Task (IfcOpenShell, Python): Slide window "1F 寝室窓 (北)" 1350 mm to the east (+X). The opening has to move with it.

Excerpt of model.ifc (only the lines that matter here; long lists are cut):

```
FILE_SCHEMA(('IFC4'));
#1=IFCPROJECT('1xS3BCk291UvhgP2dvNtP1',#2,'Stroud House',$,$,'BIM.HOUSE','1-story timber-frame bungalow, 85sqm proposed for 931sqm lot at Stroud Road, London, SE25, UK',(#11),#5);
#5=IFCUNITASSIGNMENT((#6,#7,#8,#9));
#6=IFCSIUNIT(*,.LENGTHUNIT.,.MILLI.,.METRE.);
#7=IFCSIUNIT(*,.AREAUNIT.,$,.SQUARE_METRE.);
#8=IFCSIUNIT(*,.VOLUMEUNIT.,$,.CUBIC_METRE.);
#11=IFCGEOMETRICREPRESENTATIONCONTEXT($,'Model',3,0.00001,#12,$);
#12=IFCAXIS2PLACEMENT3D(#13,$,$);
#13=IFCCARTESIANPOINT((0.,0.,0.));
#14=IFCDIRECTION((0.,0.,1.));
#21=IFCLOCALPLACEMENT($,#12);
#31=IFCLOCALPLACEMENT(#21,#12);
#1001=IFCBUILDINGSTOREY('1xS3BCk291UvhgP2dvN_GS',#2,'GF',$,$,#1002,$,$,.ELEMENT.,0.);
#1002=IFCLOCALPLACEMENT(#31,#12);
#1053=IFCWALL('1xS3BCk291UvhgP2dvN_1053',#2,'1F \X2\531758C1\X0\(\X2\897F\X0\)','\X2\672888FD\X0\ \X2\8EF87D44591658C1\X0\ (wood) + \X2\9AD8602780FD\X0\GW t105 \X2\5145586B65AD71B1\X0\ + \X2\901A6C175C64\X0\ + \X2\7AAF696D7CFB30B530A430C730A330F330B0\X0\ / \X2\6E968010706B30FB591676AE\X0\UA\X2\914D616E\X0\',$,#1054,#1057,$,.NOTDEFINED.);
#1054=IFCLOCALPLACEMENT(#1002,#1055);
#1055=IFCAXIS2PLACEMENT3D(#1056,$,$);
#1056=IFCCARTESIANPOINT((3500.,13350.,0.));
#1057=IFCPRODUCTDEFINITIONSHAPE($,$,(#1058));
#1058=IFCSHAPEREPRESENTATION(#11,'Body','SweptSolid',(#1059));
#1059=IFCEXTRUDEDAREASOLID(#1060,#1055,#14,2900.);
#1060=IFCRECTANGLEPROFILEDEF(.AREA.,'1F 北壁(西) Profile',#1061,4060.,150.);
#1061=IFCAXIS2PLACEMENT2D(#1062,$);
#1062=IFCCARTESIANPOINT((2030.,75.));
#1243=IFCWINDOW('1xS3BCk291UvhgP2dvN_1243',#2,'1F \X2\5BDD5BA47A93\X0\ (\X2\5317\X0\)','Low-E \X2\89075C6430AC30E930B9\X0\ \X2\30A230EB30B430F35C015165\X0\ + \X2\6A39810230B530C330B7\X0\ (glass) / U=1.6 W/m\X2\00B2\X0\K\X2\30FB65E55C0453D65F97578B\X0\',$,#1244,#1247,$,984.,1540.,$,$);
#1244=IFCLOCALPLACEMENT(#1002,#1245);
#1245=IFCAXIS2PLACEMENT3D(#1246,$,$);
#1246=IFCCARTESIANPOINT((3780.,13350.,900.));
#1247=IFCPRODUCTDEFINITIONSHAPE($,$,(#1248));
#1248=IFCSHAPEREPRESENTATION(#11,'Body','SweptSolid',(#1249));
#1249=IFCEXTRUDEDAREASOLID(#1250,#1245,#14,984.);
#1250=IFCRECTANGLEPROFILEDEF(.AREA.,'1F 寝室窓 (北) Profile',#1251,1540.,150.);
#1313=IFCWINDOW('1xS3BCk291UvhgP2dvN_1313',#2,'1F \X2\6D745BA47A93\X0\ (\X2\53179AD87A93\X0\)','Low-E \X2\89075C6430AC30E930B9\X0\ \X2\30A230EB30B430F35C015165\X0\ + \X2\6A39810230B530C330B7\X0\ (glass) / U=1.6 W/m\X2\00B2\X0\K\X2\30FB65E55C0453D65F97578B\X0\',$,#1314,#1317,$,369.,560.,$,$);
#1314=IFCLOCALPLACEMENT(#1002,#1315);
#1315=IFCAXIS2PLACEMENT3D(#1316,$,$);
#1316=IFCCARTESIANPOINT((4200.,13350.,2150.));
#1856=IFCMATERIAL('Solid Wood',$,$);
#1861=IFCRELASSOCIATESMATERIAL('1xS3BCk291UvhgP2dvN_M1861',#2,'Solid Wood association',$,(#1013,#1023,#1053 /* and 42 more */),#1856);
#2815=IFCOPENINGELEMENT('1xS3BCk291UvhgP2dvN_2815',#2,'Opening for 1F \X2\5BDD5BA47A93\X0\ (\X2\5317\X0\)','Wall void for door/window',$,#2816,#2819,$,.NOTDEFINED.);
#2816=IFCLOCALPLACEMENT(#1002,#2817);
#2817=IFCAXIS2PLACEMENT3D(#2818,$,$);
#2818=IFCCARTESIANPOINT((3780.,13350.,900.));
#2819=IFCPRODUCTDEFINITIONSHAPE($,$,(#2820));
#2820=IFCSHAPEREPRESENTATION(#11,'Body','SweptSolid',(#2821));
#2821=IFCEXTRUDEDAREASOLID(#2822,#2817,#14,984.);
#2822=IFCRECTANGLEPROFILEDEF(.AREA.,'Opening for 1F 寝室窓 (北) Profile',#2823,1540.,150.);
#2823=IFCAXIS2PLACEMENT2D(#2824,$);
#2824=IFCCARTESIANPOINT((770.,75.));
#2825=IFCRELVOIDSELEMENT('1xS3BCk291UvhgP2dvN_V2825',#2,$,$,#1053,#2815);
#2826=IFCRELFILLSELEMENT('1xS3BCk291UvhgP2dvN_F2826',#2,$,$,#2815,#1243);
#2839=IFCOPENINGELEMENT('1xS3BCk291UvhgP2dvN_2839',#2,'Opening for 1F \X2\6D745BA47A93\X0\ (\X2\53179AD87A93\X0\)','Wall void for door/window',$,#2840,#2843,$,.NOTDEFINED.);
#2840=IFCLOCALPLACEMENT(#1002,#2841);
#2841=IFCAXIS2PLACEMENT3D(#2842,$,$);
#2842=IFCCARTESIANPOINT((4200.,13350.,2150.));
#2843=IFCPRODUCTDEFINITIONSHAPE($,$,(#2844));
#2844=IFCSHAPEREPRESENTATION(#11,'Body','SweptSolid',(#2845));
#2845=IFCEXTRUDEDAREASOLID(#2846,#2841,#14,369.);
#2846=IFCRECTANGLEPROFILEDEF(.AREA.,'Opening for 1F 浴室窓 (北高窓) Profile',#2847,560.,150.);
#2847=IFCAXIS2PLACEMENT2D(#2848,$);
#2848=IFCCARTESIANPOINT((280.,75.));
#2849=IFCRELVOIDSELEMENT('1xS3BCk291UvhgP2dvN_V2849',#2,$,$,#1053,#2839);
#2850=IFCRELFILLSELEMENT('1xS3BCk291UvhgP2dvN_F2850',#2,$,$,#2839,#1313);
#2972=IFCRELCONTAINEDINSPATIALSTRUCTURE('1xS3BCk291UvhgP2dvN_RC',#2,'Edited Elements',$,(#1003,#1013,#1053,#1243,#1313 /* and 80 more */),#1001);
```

```python
import ifcopenshell
import ifcopenshell.api.geometry
import ifcopenshell.util.placement
import ifcopenshell.util.unit

model = ifcopenshell.open("model.ifc")
unit_scale = ifcopenshell.util.unit.calculate_unit_scale(model)

window = model.by_guid("1xS3BCk291UvhgP2dvN_1243")
opening = window.FillsVoids[0].RelatingOpeningElement
wall = opening.VoidsElements[0].RelatingBuildingElement

wall_matrix = ifcopenshell.util.placement.get_local_placement(wall.ObjectPlacement)
shift = wall_matrix[:3, 0] * 1.35 / unit_scale
before = ifcopenshell.util.placement.get_local_placement(window.ObjectPlacement)[:3, 3].copy()

# The window is not placed relative to its opening, so move both.
for product in (opening, window):
    matrix = ifcopenshell.util.placement.get_local_placement(product.ObjectPlacement)
    matrix[:3, 3] += shift
    ifcopenshell.api.geometry.edit_object_placement(model, product=product, matrix=matrix, is_si=False)

after = ifcopenshell.util.placement.get_local_placement(window.ObjectPlacement)[:3, 3]
print("window moved by", (after - before).round(3) + 0.0)

model.write("model_rev.ifc")
```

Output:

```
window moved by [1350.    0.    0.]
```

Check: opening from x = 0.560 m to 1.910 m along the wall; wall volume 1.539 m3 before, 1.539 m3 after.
